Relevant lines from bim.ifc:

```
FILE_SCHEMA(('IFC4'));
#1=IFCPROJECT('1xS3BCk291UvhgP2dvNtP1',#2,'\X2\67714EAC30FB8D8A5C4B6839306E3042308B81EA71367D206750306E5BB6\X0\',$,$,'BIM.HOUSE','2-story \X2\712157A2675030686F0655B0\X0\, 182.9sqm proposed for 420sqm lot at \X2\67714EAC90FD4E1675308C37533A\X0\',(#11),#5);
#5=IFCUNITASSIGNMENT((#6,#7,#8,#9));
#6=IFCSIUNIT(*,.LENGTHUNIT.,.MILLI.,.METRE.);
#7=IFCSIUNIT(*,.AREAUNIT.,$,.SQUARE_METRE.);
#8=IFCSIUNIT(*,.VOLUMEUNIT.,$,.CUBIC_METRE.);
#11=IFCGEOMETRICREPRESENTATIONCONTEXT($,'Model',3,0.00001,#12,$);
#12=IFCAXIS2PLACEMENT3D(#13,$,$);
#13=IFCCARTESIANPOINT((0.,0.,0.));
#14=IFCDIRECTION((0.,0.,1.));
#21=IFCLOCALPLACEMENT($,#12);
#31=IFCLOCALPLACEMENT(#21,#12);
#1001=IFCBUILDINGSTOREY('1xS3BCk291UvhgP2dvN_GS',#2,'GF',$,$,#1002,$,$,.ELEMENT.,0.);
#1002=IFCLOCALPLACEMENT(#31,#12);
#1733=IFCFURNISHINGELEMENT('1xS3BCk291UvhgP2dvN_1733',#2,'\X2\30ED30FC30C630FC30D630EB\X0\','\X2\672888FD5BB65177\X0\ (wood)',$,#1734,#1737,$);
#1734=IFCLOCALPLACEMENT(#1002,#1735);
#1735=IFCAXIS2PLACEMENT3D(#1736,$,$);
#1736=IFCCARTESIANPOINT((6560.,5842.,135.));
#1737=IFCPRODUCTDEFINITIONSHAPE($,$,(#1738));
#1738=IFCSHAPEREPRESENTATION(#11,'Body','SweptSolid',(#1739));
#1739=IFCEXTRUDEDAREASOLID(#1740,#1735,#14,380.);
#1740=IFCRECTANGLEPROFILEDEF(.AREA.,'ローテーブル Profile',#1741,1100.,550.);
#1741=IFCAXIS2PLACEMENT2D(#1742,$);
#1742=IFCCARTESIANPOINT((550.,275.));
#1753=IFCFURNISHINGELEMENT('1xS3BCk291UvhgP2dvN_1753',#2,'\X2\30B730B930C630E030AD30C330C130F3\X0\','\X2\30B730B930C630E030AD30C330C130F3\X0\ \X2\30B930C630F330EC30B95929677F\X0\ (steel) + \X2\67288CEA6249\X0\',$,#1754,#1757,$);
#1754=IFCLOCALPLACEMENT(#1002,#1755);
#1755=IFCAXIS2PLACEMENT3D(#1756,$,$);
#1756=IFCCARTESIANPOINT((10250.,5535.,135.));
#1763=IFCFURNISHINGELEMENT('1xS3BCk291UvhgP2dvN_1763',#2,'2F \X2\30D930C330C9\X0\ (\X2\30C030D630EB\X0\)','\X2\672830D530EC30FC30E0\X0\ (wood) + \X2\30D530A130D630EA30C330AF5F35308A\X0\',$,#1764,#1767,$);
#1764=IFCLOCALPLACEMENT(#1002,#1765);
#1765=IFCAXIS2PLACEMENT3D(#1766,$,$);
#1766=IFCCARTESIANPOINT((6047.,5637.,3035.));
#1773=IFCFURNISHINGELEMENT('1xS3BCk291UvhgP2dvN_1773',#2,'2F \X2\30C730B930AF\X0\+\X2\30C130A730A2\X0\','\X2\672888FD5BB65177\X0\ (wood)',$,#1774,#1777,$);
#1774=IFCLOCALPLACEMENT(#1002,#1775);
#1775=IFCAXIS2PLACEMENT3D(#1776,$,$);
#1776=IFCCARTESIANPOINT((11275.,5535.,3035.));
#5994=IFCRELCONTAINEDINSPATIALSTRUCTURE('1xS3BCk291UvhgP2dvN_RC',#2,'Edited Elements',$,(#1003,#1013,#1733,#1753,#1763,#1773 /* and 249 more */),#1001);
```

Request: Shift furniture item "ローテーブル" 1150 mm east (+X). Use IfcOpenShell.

```python
import ifcopenshell
import ifcopenshell.api.geometry
import ifcopenshell.util.placement
import ifcopenshell.util.unit

model = ifcopenshell.open("bim.ifc")
unit_scale = ifcopenshell.util.unit.calculate_unit_scale(model)

item = model.by_guid("1xS3BCk291UvhgP2dvN_1733")
matrix = ifcopenshell.util.placement.get_local_placement(item.ObjectPlacement)
matrix[0, 3] += 1.15 / unit_scale
ifcopenshell.api.geometry.edit_object_placement(model, product=item, matrix=matrix, is_si=False)

print(ifcopenshell.util.placement.get_local_placement(item.ObjectPlacement).round(3) + 0.0)

model.write("bim-out.ifc")
```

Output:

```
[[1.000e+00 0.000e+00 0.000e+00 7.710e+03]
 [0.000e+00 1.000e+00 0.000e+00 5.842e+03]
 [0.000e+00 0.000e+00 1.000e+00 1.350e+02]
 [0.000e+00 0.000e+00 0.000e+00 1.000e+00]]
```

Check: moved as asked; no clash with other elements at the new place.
